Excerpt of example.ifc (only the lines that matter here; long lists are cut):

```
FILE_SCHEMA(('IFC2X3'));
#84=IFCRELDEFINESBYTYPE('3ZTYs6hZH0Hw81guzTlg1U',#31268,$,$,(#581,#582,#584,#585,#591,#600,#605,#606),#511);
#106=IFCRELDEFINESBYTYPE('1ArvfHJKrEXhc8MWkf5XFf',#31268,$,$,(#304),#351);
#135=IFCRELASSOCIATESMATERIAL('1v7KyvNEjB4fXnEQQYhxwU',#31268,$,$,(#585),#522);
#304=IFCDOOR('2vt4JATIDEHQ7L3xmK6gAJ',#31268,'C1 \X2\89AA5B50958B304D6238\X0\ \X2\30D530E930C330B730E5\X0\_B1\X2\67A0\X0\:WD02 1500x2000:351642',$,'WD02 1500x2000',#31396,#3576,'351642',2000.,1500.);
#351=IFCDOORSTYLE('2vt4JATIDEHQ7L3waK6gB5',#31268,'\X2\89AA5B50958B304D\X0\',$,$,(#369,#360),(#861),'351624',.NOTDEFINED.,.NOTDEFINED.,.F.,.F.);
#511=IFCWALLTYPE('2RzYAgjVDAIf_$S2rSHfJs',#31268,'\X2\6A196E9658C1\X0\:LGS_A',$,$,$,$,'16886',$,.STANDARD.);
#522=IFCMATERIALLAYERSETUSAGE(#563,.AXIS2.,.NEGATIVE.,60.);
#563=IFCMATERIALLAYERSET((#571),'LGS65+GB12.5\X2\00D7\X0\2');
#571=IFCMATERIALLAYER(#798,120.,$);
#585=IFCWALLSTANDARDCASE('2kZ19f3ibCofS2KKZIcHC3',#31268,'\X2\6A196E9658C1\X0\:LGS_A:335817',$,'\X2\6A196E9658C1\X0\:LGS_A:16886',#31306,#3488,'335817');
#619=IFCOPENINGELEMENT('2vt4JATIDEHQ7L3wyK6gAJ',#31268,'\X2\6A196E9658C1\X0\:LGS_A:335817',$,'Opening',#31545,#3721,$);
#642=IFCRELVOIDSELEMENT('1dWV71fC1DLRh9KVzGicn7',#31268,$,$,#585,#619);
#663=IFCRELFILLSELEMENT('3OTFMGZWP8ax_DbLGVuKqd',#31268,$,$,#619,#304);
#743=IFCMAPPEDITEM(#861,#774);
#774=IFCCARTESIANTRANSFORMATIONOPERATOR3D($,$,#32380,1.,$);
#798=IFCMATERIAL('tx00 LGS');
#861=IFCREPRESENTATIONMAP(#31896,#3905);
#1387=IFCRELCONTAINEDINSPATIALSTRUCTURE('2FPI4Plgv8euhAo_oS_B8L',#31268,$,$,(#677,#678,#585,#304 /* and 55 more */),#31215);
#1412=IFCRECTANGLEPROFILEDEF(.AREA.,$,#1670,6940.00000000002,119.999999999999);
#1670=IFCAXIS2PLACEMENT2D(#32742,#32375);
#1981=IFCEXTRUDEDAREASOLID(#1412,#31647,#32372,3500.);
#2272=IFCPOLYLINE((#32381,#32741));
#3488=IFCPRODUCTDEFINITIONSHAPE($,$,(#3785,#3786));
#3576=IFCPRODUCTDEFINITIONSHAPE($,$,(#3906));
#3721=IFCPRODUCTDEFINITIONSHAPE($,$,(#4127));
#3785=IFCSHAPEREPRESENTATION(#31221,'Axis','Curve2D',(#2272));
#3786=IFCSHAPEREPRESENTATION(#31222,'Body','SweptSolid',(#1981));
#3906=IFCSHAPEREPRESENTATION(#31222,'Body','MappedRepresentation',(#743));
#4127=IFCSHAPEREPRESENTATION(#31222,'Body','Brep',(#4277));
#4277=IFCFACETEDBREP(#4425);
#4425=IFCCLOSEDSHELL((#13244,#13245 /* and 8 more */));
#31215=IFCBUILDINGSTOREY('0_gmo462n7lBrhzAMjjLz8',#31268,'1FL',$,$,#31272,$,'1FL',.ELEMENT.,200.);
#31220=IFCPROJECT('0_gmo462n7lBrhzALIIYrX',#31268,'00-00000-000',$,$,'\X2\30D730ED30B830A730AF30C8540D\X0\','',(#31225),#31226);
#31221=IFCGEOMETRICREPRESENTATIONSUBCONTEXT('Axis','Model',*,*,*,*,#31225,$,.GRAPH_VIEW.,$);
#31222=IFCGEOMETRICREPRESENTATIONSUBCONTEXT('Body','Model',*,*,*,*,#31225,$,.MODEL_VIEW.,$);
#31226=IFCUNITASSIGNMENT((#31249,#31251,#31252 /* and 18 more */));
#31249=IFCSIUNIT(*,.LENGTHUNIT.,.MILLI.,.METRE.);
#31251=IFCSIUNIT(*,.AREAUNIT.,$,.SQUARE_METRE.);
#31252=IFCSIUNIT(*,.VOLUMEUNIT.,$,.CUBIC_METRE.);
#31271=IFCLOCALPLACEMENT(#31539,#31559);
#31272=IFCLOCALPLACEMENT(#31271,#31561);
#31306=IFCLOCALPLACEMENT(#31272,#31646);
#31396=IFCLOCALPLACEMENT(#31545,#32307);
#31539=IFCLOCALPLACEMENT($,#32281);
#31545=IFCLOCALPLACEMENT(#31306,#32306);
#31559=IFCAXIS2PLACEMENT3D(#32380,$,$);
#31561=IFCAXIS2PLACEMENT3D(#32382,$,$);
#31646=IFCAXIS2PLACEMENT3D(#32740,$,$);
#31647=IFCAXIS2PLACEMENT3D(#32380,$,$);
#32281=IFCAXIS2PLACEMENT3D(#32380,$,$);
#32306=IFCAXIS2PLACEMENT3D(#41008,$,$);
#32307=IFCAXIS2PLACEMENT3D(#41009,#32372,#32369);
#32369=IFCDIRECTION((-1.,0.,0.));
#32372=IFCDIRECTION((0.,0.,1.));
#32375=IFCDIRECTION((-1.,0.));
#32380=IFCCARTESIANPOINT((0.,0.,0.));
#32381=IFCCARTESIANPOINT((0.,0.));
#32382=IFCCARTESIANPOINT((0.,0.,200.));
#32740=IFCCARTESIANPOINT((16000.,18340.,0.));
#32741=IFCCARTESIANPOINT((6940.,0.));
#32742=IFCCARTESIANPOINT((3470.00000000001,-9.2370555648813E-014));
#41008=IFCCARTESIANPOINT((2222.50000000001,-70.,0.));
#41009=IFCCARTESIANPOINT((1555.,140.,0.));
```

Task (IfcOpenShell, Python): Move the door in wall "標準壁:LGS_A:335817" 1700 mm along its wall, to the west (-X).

```python
import ifcopenshell
import ifcopenshell.api.geometry
import ifcopenshell.util.placement

model = ifcopenshell.open("example.ifc")

door = model.by_guid("2vt4JATIDEHQ7L3xmK6gAJ")
opening = door.FillsVoids[0].RelatingOpeningElement
wall = opening.VoidsElements[0].RelatingBuildingElement

wall_matrix = ifcopenshell.util.placement.get_local_placement(wall.ObjectPlacement)
shift = wall_matrix[:3, 0] * -1700.0
before = ifcopenshell.util.placement.get_local_placement(door.ObjectPlacement)[:3, 3].copy()

# The door is placed relative to its opening, so it follows when the opening moves.
matrix = ifcopenshell.util.placement.get_local_placement(opening.ObjectPlacement)
matrix[:3, 3] += shift
ifcopenshell.api.geometry.edit_object_placement(
    model, product=opening, matrix=matrix, is_si=False, should_transform_children=True
)

after = ifcopenshell.util.placement.get_local_placement(door.ObjectPlacement)[:3, 3]
print("door moved by", (after - before).round(3) + 0.0)

model.write("example-out.ifc")
```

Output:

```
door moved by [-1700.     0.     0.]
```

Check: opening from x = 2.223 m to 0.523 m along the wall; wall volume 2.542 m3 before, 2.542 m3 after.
